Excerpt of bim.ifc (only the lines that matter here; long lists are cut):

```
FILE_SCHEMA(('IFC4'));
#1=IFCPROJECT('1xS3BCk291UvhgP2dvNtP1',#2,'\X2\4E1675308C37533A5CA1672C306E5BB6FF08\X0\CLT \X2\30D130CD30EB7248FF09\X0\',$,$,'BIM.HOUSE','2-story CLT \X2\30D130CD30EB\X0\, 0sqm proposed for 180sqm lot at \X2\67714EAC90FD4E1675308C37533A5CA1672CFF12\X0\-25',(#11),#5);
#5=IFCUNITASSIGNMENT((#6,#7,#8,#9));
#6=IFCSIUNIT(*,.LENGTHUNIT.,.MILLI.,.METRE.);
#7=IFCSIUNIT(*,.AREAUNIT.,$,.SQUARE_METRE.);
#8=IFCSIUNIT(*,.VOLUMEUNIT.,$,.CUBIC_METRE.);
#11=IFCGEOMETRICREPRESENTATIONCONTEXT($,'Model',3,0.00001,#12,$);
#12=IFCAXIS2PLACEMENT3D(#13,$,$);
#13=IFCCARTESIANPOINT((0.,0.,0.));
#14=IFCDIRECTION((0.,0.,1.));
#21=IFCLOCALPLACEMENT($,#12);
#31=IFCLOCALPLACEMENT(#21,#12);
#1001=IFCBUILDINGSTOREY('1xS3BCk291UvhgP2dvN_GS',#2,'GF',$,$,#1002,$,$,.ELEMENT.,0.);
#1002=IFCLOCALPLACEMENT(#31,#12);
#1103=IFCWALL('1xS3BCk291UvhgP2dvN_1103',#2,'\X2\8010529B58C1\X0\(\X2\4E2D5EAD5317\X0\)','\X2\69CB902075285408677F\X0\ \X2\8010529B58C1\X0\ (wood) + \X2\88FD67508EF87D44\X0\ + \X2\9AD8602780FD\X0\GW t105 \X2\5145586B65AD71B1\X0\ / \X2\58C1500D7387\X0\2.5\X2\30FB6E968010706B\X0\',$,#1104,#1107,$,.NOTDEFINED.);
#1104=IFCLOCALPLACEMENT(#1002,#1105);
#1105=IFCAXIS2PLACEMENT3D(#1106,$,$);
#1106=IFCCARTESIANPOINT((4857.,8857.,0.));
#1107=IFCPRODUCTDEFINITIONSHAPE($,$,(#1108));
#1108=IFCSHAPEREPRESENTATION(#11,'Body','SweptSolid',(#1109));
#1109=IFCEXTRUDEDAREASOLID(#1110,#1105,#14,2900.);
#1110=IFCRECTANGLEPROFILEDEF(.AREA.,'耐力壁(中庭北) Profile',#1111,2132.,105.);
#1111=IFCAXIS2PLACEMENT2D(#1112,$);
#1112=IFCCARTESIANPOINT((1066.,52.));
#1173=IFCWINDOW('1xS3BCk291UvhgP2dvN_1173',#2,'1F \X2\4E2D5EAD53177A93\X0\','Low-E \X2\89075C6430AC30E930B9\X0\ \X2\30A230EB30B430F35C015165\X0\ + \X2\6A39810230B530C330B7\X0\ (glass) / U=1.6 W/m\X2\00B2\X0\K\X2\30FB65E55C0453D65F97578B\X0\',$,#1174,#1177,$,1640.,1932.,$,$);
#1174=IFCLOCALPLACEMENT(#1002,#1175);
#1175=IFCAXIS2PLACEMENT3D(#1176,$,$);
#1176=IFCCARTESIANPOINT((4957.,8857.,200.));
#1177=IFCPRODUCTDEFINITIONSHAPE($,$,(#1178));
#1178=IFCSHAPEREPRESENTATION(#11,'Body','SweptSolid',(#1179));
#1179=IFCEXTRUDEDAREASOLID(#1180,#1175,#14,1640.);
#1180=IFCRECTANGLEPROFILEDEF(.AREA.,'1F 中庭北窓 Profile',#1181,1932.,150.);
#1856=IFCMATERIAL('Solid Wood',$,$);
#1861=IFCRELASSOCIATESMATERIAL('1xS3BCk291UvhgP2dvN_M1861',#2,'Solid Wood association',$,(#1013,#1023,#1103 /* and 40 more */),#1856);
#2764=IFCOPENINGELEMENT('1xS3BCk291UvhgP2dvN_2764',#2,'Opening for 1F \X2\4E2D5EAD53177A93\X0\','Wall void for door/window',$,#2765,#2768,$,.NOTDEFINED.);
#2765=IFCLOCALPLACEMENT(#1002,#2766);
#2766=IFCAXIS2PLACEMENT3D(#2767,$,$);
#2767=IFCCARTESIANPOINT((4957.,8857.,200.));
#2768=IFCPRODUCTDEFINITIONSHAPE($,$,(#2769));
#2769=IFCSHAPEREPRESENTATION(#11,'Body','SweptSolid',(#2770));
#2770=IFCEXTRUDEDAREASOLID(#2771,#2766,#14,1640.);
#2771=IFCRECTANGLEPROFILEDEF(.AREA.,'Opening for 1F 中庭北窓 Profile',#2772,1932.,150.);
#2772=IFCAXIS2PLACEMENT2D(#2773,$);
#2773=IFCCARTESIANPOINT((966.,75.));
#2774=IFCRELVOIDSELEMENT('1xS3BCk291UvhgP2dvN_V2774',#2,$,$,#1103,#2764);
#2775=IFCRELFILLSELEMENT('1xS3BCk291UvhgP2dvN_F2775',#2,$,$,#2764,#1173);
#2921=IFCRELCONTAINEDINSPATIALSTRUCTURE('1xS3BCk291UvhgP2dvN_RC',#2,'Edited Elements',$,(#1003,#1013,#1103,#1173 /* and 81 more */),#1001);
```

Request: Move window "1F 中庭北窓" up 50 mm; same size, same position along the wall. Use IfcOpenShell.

```python
import numpy as np
import ifcopenshell
import ifcopenshell.api.geometry
import ifcopenshell.util.placement
import ifcopenshell.util.unit

model = ifcopenshell.open("bim.ifc")
unit_scale = ifcopenshell.util.unit.calculate_unit_scale(model)

window = model.by_guid("1xS3BCk291UvhgP2dvN_1173")
opening = window.FillsVoids[0].RelatingOpeningElement
dz = 0.05 / unit_scale

shift = np.array([0.0, 0.0, dz])
# The window is not placed relative to its opening, so move both.
for product in (opening, window):
    matrix = ifcopenshell.util.placement.get_local_placement(product.ObjectPlacement)
    matrix[:3, 3] += shift
    ifcopenshell.api.geometry.edit_object_placement(model, product=product, matrix=matrix, is_si=False)

print(f"moved by {dz * unit_scale:+.3f} m")

model.write("bim_v2.ifc")
```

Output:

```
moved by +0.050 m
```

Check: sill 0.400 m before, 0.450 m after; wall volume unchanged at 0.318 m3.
